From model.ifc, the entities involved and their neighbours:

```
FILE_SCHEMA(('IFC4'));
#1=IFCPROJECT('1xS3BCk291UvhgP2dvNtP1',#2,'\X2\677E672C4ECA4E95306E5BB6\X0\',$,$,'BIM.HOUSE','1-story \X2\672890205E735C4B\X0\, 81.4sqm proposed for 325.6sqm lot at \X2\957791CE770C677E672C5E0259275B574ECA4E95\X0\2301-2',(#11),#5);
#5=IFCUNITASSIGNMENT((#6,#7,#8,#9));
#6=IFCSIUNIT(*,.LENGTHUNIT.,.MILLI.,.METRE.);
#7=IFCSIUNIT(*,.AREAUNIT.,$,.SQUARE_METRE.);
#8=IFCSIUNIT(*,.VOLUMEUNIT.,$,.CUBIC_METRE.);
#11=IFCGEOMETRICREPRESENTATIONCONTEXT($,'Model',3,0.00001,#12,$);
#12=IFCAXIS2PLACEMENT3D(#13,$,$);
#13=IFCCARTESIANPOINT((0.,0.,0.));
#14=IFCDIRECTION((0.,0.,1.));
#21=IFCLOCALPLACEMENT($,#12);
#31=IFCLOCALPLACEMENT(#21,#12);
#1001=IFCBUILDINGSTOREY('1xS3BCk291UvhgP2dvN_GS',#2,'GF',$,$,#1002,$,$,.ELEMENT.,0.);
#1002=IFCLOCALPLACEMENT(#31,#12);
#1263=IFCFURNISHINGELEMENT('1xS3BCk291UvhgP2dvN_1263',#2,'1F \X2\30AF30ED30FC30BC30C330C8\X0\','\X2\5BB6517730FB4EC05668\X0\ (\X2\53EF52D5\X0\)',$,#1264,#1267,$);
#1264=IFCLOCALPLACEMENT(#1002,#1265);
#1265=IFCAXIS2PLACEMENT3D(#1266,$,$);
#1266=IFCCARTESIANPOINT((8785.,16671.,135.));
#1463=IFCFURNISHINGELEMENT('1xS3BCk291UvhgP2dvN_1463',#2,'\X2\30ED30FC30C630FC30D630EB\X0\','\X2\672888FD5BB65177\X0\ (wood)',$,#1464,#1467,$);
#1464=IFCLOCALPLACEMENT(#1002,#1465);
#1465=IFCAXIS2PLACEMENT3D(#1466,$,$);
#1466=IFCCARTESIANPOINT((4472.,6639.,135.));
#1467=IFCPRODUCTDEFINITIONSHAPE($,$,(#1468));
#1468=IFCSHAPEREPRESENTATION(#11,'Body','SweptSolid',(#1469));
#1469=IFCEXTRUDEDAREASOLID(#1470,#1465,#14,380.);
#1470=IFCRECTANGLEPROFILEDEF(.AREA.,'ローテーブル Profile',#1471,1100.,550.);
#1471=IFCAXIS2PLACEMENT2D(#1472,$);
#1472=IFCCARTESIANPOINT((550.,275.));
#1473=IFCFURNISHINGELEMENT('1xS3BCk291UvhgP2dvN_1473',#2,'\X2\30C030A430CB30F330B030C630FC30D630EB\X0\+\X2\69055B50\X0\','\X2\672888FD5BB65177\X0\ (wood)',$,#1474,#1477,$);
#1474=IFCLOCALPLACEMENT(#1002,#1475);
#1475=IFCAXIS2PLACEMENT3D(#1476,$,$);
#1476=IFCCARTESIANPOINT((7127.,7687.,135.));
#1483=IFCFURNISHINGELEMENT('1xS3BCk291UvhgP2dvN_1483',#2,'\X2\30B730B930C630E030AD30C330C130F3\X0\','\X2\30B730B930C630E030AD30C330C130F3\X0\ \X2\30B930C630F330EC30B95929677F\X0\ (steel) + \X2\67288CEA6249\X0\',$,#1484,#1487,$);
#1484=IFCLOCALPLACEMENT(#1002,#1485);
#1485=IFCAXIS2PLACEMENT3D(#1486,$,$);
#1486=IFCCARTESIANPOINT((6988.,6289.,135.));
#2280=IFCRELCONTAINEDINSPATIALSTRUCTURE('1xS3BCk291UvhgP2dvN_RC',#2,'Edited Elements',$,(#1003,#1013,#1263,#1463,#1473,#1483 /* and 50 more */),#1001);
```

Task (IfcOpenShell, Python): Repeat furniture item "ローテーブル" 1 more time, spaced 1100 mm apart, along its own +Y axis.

```python
import ifcopenshell
import ifcopenshell.api.geometry
import ifcopenshell.api.root
import ifcopenshell.util.element
import ifcopenshell.util.placement

model = ifcopenshell.open("model.ifc")


def reuse_history(source, copy):
    """copy_class also copies each property set's owner history, people and application; keep the originals."""
    for rel in copy.IsDefinedBy:
        if rel.is_a("IfcRelDefinesByProperties") and (history := rel.RelatingPropertyDefinition.OwnerHistory):
            rel.RelatingPropertyDefinition.OwnerHistory = source.OwnerHistory
            ifcopenshell.util.element.remove_deep2(model, history)


source = model.by_guid("1xS3BCk291UvhgP2dvN_1463")
base = ifcopenshell.util.placement.get_local_placement(source.ObjectPlacement)
step = base[:3, 1] * 1100.0

for i in range(1, 2):
    copy = ifcopenshell.api.root.copy_class(model, product=source)
    copy.Representation = ifcopenshell.util.element.copy_deep(
        model, source.Representation, exclude=["IfcGeometricRepresentationContext", "IfcRepresentationMap"]
    )
    reuse_history(source, copy)
    matrix = base.copy()
    matrix[:3, 3] += i * step
    print("added at", matrix[:3, 3].round(3) + 0.0)
    ifcopenshell.api.geometry.edit_object_placement(model, product=copy, matrix=matrix, is_si=False)

model.write("model_rev.ifc")
```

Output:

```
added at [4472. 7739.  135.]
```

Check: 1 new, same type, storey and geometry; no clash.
